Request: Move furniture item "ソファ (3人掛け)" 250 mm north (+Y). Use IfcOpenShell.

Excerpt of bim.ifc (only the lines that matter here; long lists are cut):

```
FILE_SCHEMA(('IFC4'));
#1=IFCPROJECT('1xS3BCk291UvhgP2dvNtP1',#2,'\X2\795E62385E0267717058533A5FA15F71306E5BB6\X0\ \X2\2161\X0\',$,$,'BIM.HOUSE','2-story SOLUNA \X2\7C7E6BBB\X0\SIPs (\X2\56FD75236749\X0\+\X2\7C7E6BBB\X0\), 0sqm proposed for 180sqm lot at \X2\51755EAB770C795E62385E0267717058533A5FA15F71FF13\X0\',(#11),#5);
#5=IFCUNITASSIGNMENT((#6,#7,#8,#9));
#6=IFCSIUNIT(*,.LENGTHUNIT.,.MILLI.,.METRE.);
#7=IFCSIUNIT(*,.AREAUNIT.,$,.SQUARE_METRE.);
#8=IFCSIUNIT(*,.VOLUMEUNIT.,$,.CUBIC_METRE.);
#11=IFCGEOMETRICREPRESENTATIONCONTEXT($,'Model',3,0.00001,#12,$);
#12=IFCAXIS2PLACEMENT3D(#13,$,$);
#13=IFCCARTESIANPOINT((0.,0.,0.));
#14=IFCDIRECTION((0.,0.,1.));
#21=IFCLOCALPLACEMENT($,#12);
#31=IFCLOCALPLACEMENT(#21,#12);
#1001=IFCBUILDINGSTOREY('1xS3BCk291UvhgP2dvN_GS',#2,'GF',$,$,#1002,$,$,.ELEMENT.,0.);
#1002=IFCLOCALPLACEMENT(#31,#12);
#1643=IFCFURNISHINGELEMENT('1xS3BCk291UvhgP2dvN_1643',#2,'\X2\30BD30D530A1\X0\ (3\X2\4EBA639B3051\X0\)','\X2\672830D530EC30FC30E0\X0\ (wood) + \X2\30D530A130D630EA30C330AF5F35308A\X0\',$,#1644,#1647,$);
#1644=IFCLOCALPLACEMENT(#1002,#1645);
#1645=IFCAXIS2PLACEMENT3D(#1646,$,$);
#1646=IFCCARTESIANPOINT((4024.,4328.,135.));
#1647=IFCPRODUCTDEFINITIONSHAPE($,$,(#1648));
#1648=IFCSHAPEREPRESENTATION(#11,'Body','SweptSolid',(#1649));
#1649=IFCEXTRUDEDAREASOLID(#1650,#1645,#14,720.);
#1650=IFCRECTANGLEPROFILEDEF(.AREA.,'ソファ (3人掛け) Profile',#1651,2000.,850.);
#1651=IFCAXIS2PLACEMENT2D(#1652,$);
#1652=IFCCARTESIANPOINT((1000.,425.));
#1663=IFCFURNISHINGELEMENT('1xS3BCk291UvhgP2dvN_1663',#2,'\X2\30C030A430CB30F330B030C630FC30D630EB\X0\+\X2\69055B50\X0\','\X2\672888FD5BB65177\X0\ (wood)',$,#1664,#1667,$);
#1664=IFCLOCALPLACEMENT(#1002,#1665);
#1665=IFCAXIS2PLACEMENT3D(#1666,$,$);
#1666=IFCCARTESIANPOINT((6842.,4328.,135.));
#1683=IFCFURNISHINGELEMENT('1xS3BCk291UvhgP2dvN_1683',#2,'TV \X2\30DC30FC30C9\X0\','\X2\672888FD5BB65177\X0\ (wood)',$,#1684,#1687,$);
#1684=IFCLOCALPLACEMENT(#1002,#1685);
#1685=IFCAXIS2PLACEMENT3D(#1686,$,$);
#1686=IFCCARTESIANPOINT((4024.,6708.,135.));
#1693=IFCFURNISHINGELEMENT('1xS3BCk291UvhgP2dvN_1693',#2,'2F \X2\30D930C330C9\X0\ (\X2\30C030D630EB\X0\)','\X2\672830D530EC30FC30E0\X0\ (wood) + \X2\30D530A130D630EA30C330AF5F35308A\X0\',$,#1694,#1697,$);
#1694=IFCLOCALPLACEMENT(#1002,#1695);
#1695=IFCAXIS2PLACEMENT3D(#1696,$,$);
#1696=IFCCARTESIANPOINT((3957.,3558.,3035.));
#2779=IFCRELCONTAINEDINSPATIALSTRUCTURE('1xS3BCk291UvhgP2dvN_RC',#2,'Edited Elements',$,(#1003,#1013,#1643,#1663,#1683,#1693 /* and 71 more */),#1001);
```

```python
import ifcopenshell
import ifcopenshell.api.geometry
import ifcopenshell.util.placement

model = ifcopenshell.open("bim.ifc")

item = model.by_guid("1xS3BCk291UvhgP2dvN_1643")
matrix = ifcopenshell.util.placement.get_local_placement(item.ObjectPlacement)
matrix[1, 3] += 250.0
ifcopenshell.api.geometry.edit_object_placement(model, product=item, matrix=matrix, is_si=False)

print(ifcopenshell.util.placement.get_local_placement(item.ObjectPlacement).round(3) + 0.0)

model.write("bim-out.ifc")
```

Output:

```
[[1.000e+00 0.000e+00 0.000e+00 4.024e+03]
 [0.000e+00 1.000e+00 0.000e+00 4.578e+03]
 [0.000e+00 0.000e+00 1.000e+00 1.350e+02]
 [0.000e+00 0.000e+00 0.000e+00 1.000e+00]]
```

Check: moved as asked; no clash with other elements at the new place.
